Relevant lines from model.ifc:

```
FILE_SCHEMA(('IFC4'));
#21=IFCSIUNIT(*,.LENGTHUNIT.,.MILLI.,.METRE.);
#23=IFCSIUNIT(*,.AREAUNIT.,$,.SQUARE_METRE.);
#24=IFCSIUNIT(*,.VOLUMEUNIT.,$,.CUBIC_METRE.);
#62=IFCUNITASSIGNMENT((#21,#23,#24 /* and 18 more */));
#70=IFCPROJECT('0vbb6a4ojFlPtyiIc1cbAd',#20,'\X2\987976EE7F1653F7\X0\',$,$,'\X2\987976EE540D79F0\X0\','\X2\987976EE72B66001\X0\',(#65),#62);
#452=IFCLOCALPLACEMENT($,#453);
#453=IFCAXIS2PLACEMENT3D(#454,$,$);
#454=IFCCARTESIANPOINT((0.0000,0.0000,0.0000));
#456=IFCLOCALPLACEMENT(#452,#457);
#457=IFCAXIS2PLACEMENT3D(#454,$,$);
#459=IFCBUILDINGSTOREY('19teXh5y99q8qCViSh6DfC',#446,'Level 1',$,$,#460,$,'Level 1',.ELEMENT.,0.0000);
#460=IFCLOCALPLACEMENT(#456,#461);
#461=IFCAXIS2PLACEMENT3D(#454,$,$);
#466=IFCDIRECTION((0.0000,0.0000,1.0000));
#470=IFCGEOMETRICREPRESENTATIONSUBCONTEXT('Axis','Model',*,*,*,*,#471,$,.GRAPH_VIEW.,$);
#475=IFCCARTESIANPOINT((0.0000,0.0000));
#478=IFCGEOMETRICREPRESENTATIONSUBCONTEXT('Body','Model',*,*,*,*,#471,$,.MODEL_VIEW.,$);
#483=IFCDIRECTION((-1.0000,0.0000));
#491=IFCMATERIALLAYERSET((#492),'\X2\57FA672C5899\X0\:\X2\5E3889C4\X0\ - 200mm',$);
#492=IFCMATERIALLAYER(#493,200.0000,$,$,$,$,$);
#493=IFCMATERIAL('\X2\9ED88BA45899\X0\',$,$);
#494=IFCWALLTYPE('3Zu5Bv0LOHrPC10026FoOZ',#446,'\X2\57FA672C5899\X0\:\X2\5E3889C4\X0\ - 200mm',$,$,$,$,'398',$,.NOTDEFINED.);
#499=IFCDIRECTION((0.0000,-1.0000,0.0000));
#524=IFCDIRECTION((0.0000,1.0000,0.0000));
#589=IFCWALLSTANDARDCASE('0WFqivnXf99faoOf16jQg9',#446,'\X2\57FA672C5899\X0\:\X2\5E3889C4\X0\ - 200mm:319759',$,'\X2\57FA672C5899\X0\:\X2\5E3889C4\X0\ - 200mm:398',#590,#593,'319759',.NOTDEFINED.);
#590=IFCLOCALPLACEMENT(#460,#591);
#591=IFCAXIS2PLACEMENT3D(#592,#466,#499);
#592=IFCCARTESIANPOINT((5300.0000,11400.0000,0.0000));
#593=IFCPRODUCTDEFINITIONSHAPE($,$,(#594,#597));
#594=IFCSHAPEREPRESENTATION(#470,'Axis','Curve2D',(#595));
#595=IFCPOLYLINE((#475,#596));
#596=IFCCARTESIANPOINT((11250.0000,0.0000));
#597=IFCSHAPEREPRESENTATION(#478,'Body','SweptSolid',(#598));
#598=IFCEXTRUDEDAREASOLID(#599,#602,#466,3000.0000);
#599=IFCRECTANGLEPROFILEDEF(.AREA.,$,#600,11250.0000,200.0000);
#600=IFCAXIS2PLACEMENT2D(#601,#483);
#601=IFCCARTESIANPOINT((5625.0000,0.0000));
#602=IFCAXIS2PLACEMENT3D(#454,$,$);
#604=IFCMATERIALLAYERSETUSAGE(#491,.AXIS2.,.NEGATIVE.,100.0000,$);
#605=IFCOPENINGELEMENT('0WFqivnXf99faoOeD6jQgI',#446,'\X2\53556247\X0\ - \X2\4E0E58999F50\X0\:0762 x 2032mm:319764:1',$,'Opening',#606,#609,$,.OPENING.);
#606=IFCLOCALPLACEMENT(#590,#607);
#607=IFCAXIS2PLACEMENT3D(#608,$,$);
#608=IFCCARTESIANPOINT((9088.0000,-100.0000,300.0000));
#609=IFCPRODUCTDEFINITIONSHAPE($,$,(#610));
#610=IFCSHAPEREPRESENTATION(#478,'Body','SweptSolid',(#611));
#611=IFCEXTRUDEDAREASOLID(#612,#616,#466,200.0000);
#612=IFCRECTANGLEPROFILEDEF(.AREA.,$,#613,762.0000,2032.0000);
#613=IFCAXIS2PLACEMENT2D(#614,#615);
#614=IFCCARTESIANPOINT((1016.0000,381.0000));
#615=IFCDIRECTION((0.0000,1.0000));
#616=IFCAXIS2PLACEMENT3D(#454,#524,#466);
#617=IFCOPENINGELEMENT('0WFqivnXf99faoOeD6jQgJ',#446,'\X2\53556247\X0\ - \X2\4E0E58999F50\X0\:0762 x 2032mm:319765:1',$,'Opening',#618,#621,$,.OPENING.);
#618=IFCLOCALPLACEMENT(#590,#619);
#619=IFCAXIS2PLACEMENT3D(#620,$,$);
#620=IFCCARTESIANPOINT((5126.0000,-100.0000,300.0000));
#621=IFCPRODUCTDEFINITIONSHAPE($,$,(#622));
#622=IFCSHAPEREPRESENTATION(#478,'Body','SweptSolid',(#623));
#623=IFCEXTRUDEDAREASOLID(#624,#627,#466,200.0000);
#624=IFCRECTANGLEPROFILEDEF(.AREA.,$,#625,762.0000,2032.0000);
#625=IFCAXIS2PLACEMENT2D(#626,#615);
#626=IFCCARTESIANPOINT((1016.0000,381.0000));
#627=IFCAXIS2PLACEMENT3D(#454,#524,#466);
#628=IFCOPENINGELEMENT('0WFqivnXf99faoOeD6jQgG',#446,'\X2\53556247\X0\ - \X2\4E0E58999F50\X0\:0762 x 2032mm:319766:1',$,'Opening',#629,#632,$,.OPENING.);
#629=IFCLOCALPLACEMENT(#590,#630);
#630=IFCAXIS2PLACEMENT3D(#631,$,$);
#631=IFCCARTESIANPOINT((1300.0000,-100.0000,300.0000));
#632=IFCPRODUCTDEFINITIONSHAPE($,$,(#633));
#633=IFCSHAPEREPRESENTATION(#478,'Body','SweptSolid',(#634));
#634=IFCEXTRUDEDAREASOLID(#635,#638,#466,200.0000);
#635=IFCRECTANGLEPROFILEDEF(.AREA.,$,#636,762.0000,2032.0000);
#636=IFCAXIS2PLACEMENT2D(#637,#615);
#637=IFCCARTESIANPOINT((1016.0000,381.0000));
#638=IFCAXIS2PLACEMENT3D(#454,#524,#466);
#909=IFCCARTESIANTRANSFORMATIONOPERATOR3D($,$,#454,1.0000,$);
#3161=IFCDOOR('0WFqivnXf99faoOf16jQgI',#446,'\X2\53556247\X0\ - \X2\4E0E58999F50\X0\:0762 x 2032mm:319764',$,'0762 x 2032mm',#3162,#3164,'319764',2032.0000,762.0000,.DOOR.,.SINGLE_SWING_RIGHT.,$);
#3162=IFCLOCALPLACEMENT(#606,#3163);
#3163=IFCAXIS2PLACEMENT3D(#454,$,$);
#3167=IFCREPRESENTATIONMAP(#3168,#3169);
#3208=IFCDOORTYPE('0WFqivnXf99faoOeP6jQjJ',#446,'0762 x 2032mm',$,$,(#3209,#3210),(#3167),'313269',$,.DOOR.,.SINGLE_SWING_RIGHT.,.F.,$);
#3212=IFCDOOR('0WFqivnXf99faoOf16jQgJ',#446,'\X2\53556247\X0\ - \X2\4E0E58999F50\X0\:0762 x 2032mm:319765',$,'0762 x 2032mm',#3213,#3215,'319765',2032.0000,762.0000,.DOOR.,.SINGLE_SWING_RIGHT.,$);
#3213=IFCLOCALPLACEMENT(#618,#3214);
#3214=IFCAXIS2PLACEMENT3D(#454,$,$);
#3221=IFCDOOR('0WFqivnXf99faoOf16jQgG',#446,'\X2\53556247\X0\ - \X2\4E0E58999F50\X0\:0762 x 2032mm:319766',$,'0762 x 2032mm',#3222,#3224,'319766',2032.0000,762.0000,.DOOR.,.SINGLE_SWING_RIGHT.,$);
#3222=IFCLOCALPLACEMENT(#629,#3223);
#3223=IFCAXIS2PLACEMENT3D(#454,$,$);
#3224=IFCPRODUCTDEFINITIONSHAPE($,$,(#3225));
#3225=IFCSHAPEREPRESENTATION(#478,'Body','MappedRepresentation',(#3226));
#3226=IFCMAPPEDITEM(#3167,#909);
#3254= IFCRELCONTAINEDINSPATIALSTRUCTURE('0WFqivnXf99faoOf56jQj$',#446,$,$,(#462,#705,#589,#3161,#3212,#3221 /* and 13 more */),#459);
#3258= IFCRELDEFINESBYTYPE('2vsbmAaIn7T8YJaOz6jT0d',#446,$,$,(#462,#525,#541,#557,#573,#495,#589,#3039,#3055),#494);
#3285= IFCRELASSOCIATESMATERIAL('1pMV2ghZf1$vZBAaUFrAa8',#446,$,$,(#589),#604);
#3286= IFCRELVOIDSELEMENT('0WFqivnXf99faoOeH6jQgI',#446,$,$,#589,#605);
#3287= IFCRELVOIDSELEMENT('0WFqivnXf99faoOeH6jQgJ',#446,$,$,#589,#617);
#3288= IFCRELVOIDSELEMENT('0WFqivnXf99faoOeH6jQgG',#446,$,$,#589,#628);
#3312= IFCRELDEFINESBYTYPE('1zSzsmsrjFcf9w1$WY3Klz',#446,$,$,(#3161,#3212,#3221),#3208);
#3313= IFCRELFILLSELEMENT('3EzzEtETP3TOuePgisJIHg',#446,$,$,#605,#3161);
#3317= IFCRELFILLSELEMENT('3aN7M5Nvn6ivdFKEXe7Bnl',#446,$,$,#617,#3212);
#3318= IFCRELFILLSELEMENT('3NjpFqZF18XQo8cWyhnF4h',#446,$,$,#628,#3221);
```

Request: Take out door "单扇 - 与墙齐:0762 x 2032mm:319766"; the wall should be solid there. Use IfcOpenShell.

```python
import ifcopenshell
import ifcopenshell.api.feature
import ifcopenshell.api.root
import ifcopenshell.geom
import ifcopenshell.util.shape

model = ifcopenshell.open("model.ifc")
settings = ifcopenshell.geom.settings()


def volume(element):
    """Net volume in cubic metres, openings subtracted."""
    shape = ifcopenshell.geom.create_shape(settings, element)
    return ifcopenshell.util.shape.get_volume(shape.geometry)


door = model.by_guid("0WFqivnXf99faoOf16jQgG")
opening = door.FillsVoids[0].RelatingOpeningElement
wall = opening.VoidsElements[0].RelatingBuildingElement
before = volume(wall)

ifcopenshell.api.root.remove_product(model, product=door)
ifcopenshell.api.feature.remove_feature(model, feature=opening)

after = volume(wall)

print(f"wall volume {before:.3f} -> {after:.3f} m3")

model.write("model_rev.ifc")
```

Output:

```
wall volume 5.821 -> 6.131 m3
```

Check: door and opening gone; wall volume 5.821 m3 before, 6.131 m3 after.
